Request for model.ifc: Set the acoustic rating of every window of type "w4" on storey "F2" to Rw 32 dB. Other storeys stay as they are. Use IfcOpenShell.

First a look at what the model holds.

```python
import ifcopenshell
import ifcopenshell.util.element

model = ifcopenshell.open("model.ifc")
print(model.schema)
storey = next(s for s in model.by_type("IfcBuildingStorey") if s.Name == "F2")
windows = [e for e in ifcopenshell.util.element.get_decomposition(storey) if e.is_a("IfcWindow")]
seen = {}
for e in windows:
    element_type = ifcopenshell.util.element.get_type(e)
    key = (element_type.Name if element_type != e and element_type else None, ifcopenshell.util.element.get_pset(e, "Pset_WindowCommon", "AcousticRating"))
    seen[key] = seen.get(key, 0) + 1
for (name, value), count in sorted(seen.items(), key=str):
    print(count, "x", name, "|", value)
```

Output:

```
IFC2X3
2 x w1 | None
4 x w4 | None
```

```python
import ifcopenshell
import ifcopenshell.api.pset
import ifcopenshell.util.element

model = ifcopenshell.open("model.ifc")

storey = next(s for s in model.by_type("IfcBuildingStorey") if s.Name == "F2")
windows = [e for e in ifcopenshell.util.element.get_decomposition(storey) if e.is_a("IfcWindow")]

count = 0
for e in windows:
    element_type = ifcopenshell.util.element.get_type(e)
    if element_type in (None, e) or element_type.Name != "w4":
        continue
    # add_pset returns the element's existing set when there is one.
    pset = ifcopenshell.api.pset.add_pset(model, product=e, name="Pset_WindowCommon")
    ifcopenshell.api.pset.edit_pset(model, pset=pset, properties={"AcousticRating": "Rw 32 dB"})
    count += 1

print(count, "windows updated")

model.write("model_rev.ifc")
```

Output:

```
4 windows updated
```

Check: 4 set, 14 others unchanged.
